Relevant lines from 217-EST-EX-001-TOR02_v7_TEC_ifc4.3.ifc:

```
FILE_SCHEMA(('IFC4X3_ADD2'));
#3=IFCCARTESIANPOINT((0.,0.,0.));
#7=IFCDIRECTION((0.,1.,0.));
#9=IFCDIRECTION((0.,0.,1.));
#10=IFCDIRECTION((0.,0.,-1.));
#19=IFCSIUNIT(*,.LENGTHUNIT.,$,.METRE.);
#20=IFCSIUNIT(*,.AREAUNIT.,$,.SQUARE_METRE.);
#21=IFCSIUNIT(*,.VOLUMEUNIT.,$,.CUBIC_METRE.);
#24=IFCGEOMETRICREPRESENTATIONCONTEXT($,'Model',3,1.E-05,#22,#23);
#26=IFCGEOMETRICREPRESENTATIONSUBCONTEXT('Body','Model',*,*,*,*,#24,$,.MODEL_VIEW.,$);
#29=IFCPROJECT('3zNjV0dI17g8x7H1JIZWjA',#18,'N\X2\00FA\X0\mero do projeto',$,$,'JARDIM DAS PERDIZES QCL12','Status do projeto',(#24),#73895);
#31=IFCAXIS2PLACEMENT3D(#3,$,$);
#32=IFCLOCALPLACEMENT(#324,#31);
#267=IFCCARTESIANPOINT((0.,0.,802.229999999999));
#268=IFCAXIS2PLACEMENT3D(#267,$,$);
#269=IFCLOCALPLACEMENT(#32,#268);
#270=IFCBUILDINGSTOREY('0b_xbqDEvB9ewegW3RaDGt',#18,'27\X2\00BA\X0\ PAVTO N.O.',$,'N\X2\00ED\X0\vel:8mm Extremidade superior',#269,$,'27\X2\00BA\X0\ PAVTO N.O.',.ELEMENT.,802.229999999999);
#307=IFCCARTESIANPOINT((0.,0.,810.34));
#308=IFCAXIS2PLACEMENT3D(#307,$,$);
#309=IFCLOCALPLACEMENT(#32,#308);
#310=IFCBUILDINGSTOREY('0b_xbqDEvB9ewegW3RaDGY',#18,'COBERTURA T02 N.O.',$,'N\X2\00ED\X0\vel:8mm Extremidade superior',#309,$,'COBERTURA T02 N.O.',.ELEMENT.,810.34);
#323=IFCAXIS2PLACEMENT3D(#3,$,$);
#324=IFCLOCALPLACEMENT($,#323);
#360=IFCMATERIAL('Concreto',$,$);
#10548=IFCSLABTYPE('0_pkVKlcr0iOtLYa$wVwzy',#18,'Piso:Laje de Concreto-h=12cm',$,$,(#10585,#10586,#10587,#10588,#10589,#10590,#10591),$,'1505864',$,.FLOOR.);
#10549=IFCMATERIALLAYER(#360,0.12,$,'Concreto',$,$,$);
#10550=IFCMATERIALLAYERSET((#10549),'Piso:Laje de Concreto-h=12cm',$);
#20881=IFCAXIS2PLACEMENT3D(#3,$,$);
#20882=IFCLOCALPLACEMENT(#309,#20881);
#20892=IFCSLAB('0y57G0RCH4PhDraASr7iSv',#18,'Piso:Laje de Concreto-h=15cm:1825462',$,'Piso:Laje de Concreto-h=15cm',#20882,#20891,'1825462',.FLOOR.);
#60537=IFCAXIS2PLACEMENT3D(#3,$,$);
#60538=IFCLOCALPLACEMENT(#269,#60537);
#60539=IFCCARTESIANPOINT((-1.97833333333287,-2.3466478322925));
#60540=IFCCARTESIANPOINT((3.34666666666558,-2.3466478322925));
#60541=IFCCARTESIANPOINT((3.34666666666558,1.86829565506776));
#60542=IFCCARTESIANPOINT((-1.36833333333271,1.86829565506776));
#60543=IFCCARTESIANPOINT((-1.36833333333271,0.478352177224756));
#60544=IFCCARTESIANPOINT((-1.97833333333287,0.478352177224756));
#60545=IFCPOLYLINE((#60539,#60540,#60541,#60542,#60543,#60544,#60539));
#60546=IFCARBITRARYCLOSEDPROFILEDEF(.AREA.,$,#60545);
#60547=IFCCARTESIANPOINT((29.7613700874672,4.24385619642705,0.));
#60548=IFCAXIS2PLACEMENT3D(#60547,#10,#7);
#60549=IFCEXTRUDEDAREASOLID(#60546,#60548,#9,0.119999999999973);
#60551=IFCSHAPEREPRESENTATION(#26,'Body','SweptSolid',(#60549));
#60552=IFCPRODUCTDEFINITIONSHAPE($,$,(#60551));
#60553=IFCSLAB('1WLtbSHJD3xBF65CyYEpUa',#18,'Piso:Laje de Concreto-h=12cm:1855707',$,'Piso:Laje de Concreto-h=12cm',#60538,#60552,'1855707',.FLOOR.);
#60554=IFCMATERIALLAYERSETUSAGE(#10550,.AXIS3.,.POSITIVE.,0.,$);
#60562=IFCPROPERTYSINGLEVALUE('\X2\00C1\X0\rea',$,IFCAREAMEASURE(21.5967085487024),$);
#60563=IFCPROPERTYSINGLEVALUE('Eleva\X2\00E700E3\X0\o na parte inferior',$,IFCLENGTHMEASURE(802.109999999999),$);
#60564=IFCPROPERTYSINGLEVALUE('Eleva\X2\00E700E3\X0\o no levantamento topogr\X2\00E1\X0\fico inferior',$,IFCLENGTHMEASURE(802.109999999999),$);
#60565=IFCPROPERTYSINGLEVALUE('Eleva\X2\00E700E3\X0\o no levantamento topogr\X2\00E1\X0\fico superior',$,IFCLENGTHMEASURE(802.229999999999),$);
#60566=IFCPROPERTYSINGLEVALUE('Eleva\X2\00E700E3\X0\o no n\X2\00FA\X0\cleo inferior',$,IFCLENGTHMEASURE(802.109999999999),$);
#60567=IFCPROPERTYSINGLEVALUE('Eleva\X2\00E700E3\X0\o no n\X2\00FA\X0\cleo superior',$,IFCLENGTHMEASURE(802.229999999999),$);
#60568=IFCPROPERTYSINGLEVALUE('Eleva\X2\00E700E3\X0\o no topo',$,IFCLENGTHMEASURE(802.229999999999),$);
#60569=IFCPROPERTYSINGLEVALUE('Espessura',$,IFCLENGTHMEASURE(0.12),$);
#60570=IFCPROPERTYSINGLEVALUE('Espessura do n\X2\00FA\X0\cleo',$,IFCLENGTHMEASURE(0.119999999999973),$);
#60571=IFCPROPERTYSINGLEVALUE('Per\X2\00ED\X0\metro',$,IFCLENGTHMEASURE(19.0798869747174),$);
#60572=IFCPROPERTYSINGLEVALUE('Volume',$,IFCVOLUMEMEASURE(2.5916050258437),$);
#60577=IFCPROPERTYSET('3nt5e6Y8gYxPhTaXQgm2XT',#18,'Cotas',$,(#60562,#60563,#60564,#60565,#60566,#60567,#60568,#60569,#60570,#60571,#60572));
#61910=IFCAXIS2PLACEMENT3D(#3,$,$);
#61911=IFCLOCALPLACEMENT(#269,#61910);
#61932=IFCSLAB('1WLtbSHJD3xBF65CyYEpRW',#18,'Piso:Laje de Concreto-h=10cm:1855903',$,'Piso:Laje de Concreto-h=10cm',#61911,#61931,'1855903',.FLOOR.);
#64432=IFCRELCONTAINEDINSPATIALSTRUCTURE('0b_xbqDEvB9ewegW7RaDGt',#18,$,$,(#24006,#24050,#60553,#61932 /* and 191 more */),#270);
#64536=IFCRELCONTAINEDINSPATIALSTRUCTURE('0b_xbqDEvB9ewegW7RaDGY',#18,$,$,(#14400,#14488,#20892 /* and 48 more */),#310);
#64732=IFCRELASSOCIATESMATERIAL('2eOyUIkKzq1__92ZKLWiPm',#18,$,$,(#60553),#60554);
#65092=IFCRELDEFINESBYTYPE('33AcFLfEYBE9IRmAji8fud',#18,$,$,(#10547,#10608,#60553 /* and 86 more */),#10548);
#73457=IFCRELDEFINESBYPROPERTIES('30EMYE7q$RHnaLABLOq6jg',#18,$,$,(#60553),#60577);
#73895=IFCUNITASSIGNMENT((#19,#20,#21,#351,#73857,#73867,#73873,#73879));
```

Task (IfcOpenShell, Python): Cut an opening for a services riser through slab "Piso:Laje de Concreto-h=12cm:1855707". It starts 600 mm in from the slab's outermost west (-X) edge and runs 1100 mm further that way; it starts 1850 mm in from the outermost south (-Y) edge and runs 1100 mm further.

```python
import numpy as np
import ifcopenshell
import ifcopenshell.api.feature
import ifcopenshell.api.geometry
import ifcopenshell.api.pset
import ifcopenshell.api.root
import ifcopenshell.geom
import ifcopenshell.util.element
import ifcopenshell.util.placement
import ifcopenshell.util.representation
import ifcopenshell.util.shape
import ifcopenshell.util.unit

model = ifcopenshell.open("217-EST-EX-001-TOR02_v7_TEC_ifc4.3.ifc")
unit_scale = ifcopenshell.util.unit.calculate_unit_scale(model)
area_scale = ifcopenshell.util.unit.calculate_unit_scale(model, "AREAUNIT")
volume_scale = ifcopenshell.util.unit.calculate_unit_scale(model, "VOLUMEUNIT")
settings = ifcopenshell.geom.settings()


def volume(element):
    """Net volume in cubic metres, openings subtracted."""
    shape = ifcopenshell.geom.create_shape(settings, element)
    return ifcopenshell.util.shape.get_volume(shape.geometry)


slab = model.by_id(60553)
before = volume(slab)

# Extent in the slab's own axes, in metres. The edges named are its -X and -Y sides.
slab_shape = ifcopenshell.geom.create_shape(settings, slab)
vertices = ifcopenshell.util.shape.get_vertices(slab_shape.geometry)
x_min, y_min, bottom = vertices.min(axis=0)
top = vertices[:, 2].max()

opening = ifcopenshell.api.root.create_entity(model, ifc_class="IfcOpeningElement", name="Services riser opening", predefined_type="OPENING")
context = ifcopenshell.util.representation.get_context(model, "Model", "Body", "MODEL_VIEW")
width, depth = 1.1, 1.1
outline = [(0.0, 0.0), (width, 0.0), (width, depth), (0.0, depth), (0.0, 0.0)]
# Overshoot both faces by 50 mm so the cut is clean.
shape = ifcopenshell.api.geometry.add_slab_representation(
    model, context=context, depth=top - bottom + 0.1, polyline=outline
)
ifcopenshell.api.geometry.assign_representation(model, product=opening, representation=shape)

matrix = ifcopenshell.util.placement.get_local_placement(slab.ObjectPlacement)
matrix[:, 3] = matrix @ np.append(np.array([x_min + 0.6, y_min + 1.85, bottom - 0.05]) / unit_scale, 1.0)
ifcopenshell.api.geometry.edit_object_placement(model, product=opening, matrix=matrix, is_si=False)
ifcopenshell.api.feature.add_feature(model, feature=opening, element=slab)

after = volume(slab)

# Update the slab's stored quantities.
pset = model.by_id(ifcopenshell.util.element.get_pset(slab, "Cotas", should_inherit=False)["id"])
ifcopenshell.api.pset.edit_pset(model, pset=pset, properties={
    "Área": model.create_entity("IfcAreaMeasure", after / (top - bottom) / area_scale),
    "Volume": model.create_entity("IfcVolumeMeasure", after / volume_scale),
})

print(f"slab volume {before:.3f} -> {after:.3f} m3")

model.write("217-EST-EX-001-TOR02_v7_TEC_ifc4.3_updated.ifc")
```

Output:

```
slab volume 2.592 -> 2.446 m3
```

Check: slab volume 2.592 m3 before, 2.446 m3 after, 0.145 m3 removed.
